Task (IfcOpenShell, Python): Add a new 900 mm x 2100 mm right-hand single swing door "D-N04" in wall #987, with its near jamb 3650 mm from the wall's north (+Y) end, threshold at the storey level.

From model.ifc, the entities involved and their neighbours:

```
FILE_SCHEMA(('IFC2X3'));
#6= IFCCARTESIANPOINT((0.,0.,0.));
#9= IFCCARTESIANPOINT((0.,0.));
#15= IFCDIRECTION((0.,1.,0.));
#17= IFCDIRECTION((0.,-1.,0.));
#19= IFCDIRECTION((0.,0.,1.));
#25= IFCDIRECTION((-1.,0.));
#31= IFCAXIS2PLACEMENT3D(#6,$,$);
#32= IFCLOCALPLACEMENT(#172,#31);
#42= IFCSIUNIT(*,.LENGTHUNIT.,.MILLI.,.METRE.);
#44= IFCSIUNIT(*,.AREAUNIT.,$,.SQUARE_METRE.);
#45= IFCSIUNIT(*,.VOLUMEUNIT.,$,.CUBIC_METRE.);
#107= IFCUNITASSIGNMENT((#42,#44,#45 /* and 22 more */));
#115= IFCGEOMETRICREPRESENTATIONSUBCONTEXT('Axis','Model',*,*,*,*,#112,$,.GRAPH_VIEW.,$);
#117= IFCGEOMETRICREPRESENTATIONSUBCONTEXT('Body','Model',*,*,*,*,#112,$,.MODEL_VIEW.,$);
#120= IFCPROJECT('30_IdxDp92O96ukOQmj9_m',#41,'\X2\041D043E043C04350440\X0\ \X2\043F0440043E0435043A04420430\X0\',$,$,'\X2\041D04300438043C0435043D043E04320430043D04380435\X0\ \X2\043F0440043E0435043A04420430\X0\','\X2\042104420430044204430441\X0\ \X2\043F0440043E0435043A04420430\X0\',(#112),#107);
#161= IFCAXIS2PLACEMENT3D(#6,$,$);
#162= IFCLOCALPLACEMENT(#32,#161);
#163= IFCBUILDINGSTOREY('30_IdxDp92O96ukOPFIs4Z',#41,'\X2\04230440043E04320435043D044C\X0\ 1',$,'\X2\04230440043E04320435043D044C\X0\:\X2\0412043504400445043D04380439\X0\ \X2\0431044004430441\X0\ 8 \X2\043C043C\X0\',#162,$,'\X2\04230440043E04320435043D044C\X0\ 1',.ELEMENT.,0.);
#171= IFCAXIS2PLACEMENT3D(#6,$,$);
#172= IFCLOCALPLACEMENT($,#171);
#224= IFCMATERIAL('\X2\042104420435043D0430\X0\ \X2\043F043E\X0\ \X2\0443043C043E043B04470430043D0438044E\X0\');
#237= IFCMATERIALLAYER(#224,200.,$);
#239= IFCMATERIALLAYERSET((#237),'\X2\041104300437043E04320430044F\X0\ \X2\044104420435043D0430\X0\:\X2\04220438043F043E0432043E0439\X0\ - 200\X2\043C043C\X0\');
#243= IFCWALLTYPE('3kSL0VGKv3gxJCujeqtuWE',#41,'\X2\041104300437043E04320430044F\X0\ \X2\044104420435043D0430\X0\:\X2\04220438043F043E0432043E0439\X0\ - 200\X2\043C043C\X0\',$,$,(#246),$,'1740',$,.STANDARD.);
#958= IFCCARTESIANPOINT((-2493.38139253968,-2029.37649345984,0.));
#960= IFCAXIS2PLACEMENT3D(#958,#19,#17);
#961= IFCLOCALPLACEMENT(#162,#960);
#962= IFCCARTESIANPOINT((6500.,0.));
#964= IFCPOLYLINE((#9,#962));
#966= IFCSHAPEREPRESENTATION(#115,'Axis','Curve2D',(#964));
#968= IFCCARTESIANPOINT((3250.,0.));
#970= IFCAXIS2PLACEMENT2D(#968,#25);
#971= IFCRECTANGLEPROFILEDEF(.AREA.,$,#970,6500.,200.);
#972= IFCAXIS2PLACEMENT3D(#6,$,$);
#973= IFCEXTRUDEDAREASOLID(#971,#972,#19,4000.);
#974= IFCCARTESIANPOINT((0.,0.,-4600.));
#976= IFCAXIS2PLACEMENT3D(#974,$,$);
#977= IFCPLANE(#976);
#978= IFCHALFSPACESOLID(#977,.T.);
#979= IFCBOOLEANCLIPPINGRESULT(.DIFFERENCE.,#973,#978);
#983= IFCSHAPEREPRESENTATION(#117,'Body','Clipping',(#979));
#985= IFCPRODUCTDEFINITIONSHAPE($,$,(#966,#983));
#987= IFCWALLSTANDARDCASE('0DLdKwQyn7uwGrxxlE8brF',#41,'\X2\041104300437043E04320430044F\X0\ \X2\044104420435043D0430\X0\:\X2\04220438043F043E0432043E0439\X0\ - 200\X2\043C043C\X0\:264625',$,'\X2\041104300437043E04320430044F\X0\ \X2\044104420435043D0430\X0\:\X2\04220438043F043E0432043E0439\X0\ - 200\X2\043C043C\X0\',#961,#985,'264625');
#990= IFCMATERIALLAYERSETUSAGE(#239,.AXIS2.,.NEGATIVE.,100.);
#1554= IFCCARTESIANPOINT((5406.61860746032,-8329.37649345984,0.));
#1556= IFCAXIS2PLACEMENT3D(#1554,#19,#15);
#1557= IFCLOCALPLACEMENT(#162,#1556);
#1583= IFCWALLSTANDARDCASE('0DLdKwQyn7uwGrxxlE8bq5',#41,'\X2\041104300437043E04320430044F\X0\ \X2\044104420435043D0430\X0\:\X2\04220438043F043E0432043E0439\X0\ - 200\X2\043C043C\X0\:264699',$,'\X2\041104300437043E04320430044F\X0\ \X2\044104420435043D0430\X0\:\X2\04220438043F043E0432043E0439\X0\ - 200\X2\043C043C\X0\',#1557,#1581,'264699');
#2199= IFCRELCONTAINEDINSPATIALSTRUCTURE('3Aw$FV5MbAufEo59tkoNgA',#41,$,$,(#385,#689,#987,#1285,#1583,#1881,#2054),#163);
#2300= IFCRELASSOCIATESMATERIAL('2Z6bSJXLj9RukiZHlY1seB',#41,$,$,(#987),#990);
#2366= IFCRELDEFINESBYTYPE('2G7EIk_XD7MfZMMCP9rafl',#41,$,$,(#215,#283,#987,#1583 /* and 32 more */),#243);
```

```python
import numpy as np
import ifcopenshell
import ifcopenshell.api.feature
import ifcopenshell.api.geometry
import ifcopenshell.api.root
import ifcopenshell.api.spatial
import ifcopenshell.api.type
import ifcopenshell.geom
import ifcopenshell.util.element
import ifcopenshell.util.placement
import ifcopenshell.util.representation
import ifcopenshell.util.shape
import ifcopenshell.util.unit

model = ifcopenshell.open("model.ifc")
unit_scale = ifcopenshell.util.unit.calculate_unit_scale(model)
settings = ifcopenshell.geom.settings()


def volume(element):
    """Net volume in cubic metres, openings subtracted."""
    shape = ifcopenshell.geom.create_shape(settings, element)
    return ifcopenshell.util.shape.get_volume(shape.geometry)


wall = model.by_guid("0DLdKwQyn7uwGrxxlE8brF")
storey = ifcopenshell.util.element.get_container(wall, ifc_class="IfcBuildingStorey")
context = ifcopenshell.util.representation.get_context(model, "Model", "Body", "MODEL_VIEW")
before = volume(wall)

width, height, from_end, sill = 0.9, 2.1, 3.65, 0.0  # metres

# The wall runs along its own X axis, and the end named is its -X end.
wall_shape = ifcopenshell.geom.create_shape(settings, wall)
x, y, z = ifcopenshell.util.shape.get_vertices(wall_shape.geometry).T
start = x.min() + from_end
face, thickness = float(y.min()), float(y.max() - y.min())
wall_matrix = ifcopenshell.util.placement.get_local_placement(wall.ObjectPlacement)
level = ifcopenshell.util.placement.get_local_placement(storey.ObjectPlacement)[2, 3]


def in_wall(x, y):
    """Placement at x, y metres in the wall's axes, at sill height."""
    matrix = wall_matrix.copy()
    matrix[:, 3] = wall_matrix @ np.array([x / unit_scale, y / unit_scale, 0.0, 1.0])
    matrix[2, 3] = level + sill / unit_scale
    return matrix


# Opening: a box that overshoots both wall faces by 50 mm.
opening = ifcopenshell.api.root.create_entity(model, ifc_class="IfcOpeningElement")
box = ifcopenshell.api.geometry.add_wall_representation(
    model, context=context, length=width, height=height, thickness=thickness + 0.1
)
ifcopenshell.api.geometry.assign_representation(model, product=opening, representation=box)
ifcopenshell.api.geometry.edit_object_placement(model, product=opening, matrix=in_wall(start, face - 0.05), is_si=False)
ifcopenshell.api.feature.add_feature(model, feature=opening, element=wall)

door = ifcopenshell.api.root.create_entity(model, ifc_class="IfcDoor", name="D-N04")
door.OverallWidth, door.OverallHeight = width / unit_scale, height / unit_scale
body = ifcopenshell.api.geometry.add_door_representation(
    model,
    context=context,
    overall_width=door.OverallWidth,
    overall_height=door.OverallHeight,
    operation_type="SINGLE_SWING_RIGHT",
    lining_properties={"LiningDepth": thickness / unit_scale, "ThresholdDepth": thickness / unit_scale},
)
ifcopenshell.api.geometry.assign_representation(model, product=door, representation=body)
ifcopenshell.api.spatial.assign_container(model, products=[door], relating_structure=storey)
fills = ifcopenshell.api.feature.add_filling(model, opening=opening, element=door)
fills.OwnerHistory = door.OwnerHistory  # required in IFC2X3

# IFC2X3 keeps the operation on the door style.
style = ifcopenshell.api.root.create_entity(model, ifc_class="IfcDoorStyle", name="D-N04")
style.OperationType, style.ConstructionType = "SINGLE_SWING_RIGHT", "NOTDEFINED"
style.ParameterTakesPrecedence = style.Sizeable = False
ifcopenshell.api.type.assign_type(model, related_objects=[door], relating_type=style)

# The lining spans the wall, so the door starts at the wall face.
ifcopenshell.api.geometry.edit_object_placement(model, product=door, matrix=in_wall(start, face), is_si=False)

after = volume(wall)

print(f"wall volume {before:.3f} -> {after:.3f} m3")

model.write("model_edited.ifc")
```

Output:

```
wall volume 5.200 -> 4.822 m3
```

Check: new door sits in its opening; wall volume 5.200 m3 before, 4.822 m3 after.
